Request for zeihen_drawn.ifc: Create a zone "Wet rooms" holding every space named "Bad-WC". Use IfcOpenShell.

First a look at what the model holds.

```python
import ifcopenshell

model = ifcopenshell.open("zeihen_drawn.ifc")
print(model.schema)
seen = {}
for space in model.by_type("IfcSpace"):
    seen[space.LongName] = seen.get(space.LongName, 0) + 1
for name, count in sorted(seen.items(), key=str):
    print(count, "x", name)
print("zones:", [z.Name for z in model.by_type("IfcZone")][:20])
```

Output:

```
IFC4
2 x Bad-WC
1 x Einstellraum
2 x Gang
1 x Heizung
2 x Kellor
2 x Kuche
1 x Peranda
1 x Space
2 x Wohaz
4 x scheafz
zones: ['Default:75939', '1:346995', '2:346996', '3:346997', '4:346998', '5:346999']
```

```python
import ifcopenshell
import ifcopenshell.api.group
import ifcopenshell.api.root

model = ifcopenshell.open("zeihen_drawn.ifc")

names = {"Bad-WC"}
spaces = [s for s in model.by_type("IfcSpace") if s.LongName in names]

zone = ifcopenshell.api.root.create_entity(model, ifc_class="IfcZone", name="Wet rooms")
ifcopenshell.api.group.assign_group(model, products=spaces, group=zone)
print(len(spaces), "spaces in", zone.Name)

model.write("zeihen_drawn_v2.ifc")
```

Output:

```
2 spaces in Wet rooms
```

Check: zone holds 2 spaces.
